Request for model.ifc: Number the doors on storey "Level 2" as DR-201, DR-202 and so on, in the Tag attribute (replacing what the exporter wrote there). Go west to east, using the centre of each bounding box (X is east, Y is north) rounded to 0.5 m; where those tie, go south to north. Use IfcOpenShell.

First a look at what the model holds.

```python
import ifcopenshell
import ifcopenshell.util.element
import ifcopenshell.util.placement

model = ifcopenshell.open("model.ifc")
print(model.schema)
storey = next(s for s in model.by_type("IfcBuildingStorey") if s.Name == "Level 2")
doors = [e for e in ifcopenshell.util.element.get_decomposition(storey) if e.is_a("IfcDoor")]
for e in sorted(doors, key=lambda e: e.id()):
    origin = ifcopenshell.util.placement.get_local_placement(e.ObjectPlacement)[:3, 3]
    print(e.id(), e.Tag, e.Name, origin.round(2) + 0.0, sep=" | ")
```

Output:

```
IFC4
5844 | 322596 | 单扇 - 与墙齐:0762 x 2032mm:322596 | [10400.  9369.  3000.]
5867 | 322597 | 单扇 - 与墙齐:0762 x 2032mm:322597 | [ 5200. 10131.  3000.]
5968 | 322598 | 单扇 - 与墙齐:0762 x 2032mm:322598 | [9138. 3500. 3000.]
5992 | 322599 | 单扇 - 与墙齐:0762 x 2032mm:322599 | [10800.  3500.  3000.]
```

```python
import ifcopenshell
import ifcopenshell.geom
import ifcopenshell.util.element
import ifcopenshell.util.shape

model = ifcopenshell.open("model.ifc")
settings = ifcopenshell.geom.settings()
settings.set("use-world-coords", True)


def centre(element):
    shape = ifcopenshell.geom.create_shape(settings, element)
    return ifcopenshell.util.shape.get_bbox_centroid(shape.geometry)


storey = next(s for s in model.by_type("IfcBuildingStorey") if s.Name == "Level 2")
doors = [e for e in ifcopenshell.util.element.get_decomposition(storey) if e.is_a("IfcDoor")]

# Insertion points can sit at a corner or the storey origin, so sort by the geometry (in metres).
centres = {e: centre(e) for e in doors}
doors.sort(key=lambda e: (round(centres[e][0] / 0.5), centres[e][1]))

for i, e in enumerate(doors, start=1):
    number = f"DR-2{i:02d}"
    e.Tag = number
    print(e.id(), number)

model.write("model_edited.ifc")
```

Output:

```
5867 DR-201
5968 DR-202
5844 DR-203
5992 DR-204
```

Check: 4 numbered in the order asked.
